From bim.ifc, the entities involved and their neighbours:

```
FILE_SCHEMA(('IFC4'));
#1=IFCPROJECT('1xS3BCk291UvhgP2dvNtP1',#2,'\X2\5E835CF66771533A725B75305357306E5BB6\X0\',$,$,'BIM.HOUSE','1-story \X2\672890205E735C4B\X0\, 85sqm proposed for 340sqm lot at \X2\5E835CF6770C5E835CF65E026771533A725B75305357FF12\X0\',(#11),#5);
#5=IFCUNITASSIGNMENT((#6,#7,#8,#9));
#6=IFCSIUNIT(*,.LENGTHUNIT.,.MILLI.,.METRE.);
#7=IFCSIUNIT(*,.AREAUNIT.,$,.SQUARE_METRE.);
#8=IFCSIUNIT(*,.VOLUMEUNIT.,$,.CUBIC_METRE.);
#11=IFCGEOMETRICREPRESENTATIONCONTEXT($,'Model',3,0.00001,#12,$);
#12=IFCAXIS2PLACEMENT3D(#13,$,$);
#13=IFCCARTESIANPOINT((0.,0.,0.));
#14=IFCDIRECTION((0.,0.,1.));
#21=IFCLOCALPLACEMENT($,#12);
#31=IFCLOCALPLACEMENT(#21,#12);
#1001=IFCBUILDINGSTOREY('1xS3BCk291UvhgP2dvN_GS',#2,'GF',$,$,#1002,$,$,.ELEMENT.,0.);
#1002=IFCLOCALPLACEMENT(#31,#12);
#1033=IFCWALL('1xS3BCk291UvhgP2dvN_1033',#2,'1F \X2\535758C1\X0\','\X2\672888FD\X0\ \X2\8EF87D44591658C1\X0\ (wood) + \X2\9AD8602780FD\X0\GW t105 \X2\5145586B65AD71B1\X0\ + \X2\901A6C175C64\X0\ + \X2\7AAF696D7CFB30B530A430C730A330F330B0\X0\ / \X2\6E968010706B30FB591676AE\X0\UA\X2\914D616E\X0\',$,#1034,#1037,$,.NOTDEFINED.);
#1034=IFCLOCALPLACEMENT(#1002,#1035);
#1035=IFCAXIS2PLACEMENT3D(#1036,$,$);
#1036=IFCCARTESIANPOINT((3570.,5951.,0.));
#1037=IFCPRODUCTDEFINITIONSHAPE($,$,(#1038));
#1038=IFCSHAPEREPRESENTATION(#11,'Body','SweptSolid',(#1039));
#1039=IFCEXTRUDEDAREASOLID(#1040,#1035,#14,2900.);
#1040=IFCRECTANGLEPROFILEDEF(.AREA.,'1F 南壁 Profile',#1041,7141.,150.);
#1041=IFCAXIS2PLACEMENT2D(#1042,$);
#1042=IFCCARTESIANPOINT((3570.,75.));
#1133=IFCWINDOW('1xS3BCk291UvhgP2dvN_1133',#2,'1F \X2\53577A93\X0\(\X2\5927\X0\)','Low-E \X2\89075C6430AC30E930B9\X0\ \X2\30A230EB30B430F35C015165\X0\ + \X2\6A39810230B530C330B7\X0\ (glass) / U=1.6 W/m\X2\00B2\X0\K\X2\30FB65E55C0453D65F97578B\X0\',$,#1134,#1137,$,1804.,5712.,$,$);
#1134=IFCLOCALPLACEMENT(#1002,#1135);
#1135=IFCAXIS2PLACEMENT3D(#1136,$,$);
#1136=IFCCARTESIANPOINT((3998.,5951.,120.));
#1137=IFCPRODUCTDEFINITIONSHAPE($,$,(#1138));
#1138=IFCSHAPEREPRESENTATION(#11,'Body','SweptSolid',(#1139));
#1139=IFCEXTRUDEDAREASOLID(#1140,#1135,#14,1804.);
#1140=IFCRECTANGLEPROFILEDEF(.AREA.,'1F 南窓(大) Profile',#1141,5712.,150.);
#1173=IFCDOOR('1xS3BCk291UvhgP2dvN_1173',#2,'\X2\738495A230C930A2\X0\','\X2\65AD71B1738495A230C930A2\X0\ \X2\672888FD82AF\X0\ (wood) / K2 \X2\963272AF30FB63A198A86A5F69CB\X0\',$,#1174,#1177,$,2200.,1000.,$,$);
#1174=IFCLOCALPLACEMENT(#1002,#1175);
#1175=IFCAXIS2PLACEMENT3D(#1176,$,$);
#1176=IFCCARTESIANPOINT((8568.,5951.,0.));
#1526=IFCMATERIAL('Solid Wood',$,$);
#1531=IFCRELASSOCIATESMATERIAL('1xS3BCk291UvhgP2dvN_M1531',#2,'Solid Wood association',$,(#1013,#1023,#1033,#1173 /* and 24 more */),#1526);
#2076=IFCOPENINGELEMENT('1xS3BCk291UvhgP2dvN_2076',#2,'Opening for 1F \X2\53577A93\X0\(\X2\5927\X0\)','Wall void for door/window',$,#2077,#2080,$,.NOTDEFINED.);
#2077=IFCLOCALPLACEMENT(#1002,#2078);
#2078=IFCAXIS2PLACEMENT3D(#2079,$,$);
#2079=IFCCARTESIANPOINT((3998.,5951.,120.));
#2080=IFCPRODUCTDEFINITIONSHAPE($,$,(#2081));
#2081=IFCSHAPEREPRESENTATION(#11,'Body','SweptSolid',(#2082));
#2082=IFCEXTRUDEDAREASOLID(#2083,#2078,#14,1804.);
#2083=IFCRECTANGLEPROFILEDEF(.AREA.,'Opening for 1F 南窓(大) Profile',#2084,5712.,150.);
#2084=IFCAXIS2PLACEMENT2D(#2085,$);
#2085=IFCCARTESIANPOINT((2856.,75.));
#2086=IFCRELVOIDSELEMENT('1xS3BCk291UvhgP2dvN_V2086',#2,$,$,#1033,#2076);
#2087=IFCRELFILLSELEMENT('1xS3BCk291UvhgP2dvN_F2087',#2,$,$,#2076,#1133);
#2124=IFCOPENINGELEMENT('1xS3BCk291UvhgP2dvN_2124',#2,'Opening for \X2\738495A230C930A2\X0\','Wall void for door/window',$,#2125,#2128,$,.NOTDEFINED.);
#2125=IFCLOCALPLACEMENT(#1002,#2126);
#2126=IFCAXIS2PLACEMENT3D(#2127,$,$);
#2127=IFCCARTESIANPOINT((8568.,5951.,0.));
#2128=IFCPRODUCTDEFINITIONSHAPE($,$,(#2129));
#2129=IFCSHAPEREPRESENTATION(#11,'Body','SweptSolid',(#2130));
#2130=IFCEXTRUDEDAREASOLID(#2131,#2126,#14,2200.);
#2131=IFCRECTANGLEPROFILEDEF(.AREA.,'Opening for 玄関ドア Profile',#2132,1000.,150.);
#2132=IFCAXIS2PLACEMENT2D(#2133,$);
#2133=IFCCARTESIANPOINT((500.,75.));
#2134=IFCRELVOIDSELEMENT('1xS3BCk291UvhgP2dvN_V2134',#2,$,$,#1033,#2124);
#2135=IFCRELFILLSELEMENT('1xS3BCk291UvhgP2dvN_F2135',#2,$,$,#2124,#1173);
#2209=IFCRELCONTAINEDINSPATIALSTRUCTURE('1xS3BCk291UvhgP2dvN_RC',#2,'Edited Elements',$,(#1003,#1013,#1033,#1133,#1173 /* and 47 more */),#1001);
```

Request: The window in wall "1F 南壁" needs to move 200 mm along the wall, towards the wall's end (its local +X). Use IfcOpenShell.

```python
import ifcopenshell
import ifcopenshell.api.geometry
import ifcopenshell.util.placement

model = ifcopenshell.open("bim.ifc")

window = model.by_guid("1xS3BCk291UvhgP2dvN_1133")
opening = window.FillsVoids[0].RelatingOpeningElement
wall = opening.VoidsElements[0].RelatingBuildingElement

wall_matrix = ifcopenshell.util.placement.get_local_placement(wall.ObjectPlacement)
shift = wall_matrix[:3, 0] * 200.0
before = ifcopenshell.util.placement.get_local_placement(window.ObjectPlacement)[:3, 3].copy()

# The window is not placed relative to its opening, so move both.
for product in (opening, window):
    matrix = ifcopenshell.util.placement.get_local_placement(product.ObjectPlacement)
    matrix[:3, 3] += shift
    ifcopenshell.api.geometry.edit_object_placement(model, product=product, matrix=matrix, is_si=False)

after = ifcopenshell.util.placement.get_local_placement(window.ObjectPlacement)[:3, 3]
print("window moved by", (after - before).round(3) + 0.0)

model.write("bim_rev.ifc")
```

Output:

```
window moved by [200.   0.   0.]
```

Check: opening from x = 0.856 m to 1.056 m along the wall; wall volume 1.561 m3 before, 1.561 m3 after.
